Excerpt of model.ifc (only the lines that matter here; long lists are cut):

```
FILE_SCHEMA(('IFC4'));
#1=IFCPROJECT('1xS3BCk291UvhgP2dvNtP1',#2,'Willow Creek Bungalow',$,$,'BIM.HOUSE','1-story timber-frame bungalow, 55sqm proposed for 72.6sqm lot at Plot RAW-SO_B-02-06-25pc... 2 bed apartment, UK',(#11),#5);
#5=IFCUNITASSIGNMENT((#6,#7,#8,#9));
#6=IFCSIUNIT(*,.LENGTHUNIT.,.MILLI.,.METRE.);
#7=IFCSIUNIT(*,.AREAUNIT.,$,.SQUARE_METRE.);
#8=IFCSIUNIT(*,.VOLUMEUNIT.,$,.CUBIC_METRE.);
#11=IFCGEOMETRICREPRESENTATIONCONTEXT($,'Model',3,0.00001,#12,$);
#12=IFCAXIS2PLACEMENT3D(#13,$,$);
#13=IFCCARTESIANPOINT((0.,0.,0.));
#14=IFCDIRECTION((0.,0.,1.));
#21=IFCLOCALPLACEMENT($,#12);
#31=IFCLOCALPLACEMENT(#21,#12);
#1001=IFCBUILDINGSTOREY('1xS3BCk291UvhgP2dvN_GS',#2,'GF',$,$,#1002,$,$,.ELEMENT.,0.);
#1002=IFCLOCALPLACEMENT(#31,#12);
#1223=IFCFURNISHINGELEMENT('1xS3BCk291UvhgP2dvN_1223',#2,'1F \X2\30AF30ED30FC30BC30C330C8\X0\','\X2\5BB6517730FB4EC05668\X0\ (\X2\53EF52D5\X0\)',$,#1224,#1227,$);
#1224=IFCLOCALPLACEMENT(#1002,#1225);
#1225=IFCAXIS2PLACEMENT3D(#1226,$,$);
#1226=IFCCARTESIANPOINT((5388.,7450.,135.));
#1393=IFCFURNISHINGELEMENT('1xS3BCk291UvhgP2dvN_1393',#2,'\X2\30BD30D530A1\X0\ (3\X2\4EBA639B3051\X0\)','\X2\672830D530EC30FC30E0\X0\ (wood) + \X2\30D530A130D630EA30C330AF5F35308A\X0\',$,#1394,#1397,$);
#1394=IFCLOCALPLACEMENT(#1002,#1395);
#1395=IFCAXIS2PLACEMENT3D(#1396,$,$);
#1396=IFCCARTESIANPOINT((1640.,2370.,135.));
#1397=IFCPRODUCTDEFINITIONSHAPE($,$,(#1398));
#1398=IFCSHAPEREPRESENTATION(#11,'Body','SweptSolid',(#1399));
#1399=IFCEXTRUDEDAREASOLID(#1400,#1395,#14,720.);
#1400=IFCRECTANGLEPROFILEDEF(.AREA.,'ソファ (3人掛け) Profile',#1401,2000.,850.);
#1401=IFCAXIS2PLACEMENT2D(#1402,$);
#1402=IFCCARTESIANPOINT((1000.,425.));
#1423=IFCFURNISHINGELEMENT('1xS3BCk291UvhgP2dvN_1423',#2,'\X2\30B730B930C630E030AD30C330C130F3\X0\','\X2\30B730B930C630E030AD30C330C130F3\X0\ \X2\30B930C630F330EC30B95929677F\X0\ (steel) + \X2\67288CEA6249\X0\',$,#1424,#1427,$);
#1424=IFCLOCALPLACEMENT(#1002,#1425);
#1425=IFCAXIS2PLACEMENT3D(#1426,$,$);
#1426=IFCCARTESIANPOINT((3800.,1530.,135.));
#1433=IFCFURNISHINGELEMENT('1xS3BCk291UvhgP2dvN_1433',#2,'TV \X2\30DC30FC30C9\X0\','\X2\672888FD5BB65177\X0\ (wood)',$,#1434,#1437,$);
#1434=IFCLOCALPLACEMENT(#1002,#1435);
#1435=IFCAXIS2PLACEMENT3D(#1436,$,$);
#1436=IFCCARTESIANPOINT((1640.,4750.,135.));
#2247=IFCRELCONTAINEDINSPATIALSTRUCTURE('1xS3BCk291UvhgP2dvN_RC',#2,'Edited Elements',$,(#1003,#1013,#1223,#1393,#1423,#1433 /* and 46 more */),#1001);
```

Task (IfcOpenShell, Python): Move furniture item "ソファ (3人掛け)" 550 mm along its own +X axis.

```python
import ifcopenshell
import ifcopenshell.api.geometry
import ifcopenshell.util.placement

model = ifcopenshell.open("model.ifc")

item = model.by_guid("1xS3BCk291UvhgP2dvN_1393")
matrix = ifcopenshell.util.placement.get_local_placement(item.ObjectPlacement)
matrix[:3, 3] += matrix[:3, 0] * 550.0
ifcopenshell.api.geometry.edit_object_placement(model, product=item, matrix=matrix, is_si=False)

print(ifcopenshell.util.placement.get_local_placement(item.ObjectPlacement).round(3) + 0.0)

model.write("model-out.ifc")
```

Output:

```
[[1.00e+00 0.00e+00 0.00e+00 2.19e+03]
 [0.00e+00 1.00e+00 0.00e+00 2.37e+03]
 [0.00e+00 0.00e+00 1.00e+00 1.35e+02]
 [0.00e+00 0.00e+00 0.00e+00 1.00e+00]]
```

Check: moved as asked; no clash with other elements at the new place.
